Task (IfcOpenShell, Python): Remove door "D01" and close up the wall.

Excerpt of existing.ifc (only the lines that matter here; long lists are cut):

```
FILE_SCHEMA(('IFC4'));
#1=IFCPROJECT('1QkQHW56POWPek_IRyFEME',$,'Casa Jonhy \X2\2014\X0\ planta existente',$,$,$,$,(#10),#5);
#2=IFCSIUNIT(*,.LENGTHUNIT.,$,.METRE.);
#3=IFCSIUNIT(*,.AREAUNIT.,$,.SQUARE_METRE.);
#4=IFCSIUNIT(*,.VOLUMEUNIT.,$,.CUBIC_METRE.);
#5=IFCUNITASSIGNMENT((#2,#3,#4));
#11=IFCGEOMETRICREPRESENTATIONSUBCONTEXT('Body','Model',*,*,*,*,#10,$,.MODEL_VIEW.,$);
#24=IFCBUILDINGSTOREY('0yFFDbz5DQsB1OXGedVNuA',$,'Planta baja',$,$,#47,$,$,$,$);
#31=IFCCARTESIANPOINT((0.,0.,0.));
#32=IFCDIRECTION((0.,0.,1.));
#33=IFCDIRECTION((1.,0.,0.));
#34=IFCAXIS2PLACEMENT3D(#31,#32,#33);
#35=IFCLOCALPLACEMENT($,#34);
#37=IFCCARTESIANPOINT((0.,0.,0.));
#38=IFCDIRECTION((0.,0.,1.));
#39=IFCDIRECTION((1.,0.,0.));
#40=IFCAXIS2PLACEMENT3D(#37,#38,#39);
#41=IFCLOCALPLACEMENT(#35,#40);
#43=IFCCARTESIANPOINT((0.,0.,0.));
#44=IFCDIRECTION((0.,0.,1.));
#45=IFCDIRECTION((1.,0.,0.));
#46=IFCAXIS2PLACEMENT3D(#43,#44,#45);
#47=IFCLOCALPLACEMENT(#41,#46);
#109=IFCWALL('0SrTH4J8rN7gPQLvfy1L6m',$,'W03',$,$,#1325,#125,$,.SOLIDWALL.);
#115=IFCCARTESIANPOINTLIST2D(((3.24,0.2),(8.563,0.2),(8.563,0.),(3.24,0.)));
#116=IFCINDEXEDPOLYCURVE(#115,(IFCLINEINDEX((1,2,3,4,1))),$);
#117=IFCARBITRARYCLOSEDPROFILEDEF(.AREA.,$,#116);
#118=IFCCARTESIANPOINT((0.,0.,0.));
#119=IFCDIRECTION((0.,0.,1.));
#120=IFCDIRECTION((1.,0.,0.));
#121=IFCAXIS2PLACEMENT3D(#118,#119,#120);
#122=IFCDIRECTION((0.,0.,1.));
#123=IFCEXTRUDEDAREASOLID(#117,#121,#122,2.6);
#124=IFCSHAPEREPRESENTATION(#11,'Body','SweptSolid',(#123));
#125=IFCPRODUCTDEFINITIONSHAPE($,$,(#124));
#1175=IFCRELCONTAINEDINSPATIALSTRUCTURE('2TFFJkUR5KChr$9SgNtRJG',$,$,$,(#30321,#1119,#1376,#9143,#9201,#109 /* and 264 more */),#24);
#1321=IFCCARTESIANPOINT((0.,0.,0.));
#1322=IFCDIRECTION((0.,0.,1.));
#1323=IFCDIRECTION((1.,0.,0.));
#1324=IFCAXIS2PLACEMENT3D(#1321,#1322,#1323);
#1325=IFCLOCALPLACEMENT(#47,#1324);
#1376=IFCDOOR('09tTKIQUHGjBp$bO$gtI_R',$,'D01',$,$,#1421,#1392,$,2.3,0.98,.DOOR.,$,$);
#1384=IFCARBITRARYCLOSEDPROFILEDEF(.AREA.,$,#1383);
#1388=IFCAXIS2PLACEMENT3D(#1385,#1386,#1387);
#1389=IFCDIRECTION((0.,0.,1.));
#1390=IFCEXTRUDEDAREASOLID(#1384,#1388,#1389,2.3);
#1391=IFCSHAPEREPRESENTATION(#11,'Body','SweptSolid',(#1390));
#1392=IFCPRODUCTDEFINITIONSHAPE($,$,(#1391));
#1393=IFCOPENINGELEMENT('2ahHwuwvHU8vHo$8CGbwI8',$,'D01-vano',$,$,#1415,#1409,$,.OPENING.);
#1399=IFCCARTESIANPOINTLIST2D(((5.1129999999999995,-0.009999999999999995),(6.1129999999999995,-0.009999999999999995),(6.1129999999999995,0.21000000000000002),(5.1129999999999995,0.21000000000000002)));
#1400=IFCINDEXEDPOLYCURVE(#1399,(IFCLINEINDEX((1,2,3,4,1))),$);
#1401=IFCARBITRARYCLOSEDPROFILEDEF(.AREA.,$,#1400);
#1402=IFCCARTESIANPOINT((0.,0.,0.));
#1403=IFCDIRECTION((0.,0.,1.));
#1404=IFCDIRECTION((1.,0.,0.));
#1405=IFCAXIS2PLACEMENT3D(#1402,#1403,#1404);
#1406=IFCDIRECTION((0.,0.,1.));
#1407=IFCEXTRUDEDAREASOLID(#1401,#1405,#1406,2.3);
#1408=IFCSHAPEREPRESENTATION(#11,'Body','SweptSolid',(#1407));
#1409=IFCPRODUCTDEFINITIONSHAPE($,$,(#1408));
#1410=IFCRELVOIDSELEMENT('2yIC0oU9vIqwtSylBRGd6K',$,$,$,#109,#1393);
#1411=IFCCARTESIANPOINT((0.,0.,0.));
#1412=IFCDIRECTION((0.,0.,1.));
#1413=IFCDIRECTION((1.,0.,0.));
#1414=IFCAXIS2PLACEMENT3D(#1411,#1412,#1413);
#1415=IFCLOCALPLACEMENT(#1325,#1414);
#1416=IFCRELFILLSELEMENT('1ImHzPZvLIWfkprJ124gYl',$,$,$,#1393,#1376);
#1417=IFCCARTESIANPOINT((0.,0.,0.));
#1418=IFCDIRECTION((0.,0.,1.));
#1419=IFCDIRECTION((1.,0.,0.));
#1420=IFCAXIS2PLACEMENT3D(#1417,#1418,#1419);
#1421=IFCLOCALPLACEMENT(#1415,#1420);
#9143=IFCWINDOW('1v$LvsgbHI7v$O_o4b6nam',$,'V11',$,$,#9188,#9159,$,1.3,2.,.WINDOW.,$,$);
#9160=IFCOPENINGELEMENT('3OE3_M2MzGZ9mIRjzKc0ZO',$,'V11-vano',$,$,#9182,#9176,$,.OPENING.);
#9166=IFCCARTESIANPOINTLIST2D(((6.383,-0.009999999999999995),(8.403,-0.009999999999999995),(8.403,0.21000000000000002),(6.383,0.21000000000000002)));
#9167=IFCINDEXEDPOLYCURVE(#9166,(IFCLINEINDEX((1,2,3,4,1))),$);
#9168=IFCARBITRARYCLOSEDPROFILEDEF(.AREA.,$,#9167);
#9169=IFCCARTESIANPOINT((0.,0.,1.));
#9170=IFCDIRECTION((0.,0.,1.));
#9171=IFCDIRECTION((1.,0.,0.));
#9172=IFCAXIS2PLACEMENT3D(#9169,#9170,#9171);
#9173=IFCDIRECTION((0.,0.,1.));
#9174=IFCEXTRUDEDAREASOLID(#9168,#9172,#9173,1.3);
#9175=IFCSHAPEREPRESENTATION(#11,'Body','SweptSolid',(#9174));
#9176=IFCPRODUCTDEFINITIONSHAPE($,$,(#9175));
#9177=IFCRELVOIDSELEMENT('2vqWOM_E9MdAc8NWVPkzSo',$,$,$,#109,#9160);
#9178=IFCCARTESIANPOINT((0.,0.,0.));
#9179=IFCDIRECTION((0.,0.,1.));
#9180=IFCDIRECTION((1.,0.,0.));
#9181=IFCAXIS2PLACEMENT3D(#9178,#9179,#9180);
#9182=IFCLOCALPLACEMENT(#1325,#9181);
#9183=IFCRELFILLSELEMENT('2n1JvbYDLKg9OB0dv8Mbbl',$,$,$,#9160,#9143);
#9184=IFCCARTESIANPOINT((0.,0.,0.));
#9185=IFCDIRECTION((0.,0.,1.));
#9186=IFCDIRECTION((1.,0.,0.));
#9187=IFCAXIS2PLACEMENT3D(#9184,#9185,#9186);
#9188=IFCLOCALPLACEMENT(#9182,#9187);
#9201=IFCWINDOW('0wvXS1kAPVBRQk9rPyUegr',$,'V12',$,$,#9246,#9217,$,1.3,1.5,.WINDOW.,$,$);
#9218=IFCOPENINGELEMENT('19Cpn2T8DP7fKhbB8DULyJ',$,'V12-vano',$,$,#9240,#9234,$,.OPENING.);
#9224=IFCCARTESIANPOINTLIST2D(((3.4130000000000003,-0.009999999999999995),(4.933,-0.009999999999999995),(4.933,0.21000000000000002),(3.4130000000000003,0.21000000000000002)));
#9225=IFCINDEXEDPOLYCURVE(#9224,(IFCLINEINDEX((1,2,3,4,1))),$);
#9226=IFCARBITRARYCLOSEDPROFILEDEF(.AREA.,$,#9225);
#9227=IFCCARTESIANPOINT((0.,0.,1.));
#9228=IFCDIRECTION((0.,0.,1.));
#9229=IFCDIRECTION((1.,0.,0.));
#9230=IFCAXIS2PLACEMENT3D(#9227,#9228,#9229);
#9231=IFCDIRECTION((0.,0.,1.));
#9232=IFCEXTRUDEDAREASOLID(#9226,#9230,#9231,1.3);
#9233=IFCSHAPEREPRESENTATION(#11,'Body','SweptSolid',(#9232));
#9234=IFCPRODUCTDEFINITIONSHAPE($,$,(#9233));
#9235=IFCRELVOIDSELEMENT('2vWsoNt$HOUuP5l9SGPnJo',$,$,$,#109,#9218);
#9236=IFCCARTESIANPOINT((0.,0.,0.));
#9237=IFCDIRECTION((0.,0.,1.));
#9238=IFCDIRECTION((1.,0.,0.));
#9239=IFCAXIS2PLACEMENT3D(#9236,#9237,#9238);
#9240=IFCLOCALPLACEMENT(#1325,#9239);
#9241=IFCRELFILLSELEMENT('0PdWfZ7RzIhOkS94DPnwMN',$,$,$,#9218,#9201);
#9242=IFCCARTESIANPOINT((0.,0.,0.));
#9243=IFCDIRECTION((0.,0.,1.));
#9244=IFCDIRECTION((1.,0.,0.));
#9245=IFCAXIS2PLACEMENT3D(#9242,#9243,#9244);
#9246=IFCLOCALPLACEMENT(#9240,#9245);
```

```python
import ifcopenshell
import ifcopenshell.api.feature
import ifcopenshell.api.root
import ifcopenshell.geom
import ifcopenshell.util.shape

model = ifcopenshell.open("existing.ifc")
settings = ifcopenshell.geom.settings()


def volume(element):
    """Net volume in cubic metres, openings subtracted."""
    shape = ifcopenshell.geom.create_shape(settings, element)
    return ifcopenshell.util.shape.get_volume(shape.geometry)


door = model.by_guid("09tTKIQUHGjBp$bO$gtI_R")
opening = door.FillsVoids[0].RelatingOpeningElement
wall = opening.VoidsElements[0].RelatingBuildingElement
before = volume(wall)

ifcopenshell.api.root.remove_product(model, product=door)
ifcopenshell.api.feature.remove_feature(model, feature=opening)

after = volume(wall)

print(f"wall volume {before:.3f} -> {after:.3f} m3")

model.write("existing_rev.ifc")
```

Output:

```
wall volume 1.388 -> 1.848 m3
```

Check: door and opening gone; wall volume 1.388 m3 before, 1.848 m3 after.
